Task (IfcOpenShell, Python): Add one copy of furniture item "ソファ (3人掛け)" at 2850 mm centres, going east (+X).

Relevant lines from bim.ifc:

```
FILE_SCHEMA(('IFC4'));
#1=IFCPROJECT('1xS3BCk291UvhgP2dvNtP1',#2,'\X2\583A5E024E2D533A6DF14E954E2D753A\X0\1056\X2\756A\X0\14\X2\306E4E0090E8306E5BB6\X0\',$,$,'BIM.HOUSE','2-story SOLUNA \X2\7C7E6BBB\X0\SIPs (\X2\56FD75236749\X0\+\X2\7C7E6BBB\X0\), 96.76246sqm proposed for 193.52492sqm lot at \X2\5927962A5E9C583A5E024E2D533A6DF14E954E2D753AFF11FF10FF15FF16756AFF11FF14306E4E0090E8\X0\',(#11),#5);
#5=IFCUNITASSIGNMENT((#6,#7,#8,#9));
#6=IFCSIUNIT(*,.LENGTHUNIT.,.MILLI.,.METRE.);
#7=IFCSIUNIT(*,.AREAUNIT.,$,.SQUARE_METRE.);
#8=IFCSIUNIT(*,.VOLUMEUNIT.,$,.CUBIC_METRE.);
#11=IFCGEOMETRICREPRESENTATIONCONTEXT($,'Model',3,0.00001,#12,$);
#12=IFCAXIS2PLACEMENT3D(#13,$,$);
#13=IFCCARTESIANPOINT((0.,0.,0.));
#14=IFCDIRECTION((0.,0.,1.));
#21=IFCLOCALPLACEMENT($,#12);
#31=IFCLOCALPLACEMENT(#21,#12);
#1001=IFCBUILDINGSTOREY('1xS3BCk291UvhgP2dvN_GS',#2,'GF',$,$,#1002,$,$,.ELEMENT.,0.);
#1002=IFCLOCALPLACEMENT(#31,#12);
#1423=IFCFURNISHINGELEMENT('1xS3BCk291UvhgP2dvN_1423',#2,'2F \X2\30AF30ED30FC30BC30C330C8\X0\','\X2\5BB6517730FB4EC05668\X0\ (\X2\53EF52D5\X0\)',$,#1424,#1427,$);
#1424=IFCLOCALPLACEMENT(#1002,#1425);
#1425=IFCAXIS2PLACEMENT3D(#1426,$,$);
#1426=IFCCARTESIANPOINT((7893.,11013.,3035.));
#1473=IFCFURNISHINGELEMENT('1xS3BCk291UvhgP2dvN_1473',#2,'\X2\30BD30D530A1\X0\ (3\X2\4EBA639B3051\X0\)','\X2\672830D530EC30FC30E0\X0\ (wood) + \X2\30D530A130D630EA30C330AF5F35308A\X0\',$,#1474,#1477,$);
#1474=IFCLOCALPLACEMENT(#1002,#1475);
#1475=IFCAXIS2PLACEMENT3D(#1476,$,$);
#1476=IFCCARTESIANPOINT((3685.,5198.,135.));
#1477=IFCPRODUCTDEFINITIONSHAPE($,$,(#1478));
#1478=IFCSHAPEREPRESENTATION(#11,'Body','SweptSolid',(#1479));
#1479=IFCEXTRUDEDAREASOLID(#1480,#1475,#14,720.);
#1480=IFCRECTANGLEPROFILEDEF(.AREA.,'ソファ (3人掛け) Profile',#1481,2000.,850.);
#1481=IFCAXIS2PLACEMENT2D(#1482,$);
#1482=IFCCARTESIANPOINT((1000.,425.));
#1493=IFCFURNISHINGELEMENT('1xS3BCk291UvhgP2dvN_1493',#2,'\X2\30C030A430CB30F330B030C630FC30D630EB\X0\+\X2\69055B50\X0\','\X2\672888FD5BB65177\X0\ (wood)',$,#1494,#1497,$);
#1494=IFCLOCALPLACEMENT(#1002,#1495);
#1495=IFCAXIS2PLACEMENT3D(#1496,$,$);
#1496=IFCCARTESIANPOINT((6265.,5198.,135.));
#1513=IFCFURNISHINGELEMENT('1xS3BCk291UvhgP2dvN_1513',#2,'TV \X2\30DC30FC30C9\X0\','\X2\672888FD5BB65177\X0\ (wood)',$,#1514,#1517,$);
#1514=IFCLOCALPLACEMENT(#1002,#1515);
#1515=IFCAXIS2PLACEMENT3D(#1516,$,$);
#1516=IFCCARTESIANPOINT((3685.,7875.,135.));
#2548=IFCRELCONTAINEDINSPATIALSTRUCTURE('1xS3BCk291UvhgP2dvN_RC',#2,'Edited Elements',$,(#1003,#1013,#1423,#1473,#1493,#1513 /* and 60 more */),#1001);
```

```python
import numpy as np
import ifcopenshell
import ifcopenshell.api.geometry
import ifcopenshell.api.root
import ifcopenshell.util.element
import ifcopenshell.util.placement
import ifcopenshell.util.unit

model = ifcopenshell.open("bim.ifc")
unit_scale = ifcopenshell.util.unit.calculate_unit_scale(model)


def reuse_history(source, copy):
    """copy_class also copies each property set's owner history, people and application; keep the originals."""
    for rel in copy.IsDefinedBy:
        if rel.is_a("IfcRelDefinesByProperties") and (history := rel.RelatingPropertyDefinition.OwnerHistory):
            rel.RelatingPropertyDefinition.OwnerHistory = source.OwnerHistory
            ifcopenshell.util.element.remove_deep2(model, history)


source = model.by_id(1473)
base = ifcopenshell.util.placement.get_local_placement(source.ObjectPlacement)
step = np.array([1.0, 0.0, 0.0]) * 2.85 / unit_scale

for i in range(1, 2):
    copy = ifcopenshell.api.root.copy_class(model, product=source)
    copy.Representation = ifcopenshell.util.element.copy_deep(
        model, source.Representation, exclude=["IfcGeometricRepresentationContext", "IfcRepresentationMap"]
    )
    reuse_history(source, copy)
    matrix = base.copy()
    matrix[:3, 3] += i * step
    print("added at", matrix[:3, 3].round(3) + 0.0)
    ifcopenshell.api.geometry.edit_object_placement(model, product=copy, matrix=matrix, is_si=False)

model.write("bim_edited.ifc")
```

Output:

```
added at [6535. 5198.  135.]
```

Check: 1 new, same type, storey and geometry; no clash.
